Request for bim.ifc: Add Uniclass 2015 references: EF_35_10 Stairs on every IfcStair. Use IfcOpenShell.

First a look at what the model holds.

```python
import ifcopenshell

model = ifcopenshell.open("bim.ifc")
print(model.schema)
print("classifications:", [c.Name for c in model.by_type("IfcClassification")])
for ifc_class in ("IfcDoor", "IfcRoof", "IfcStair", "IfcWall", "IfcWindow"):
    print(ifc_class, len(model.by_type(ifc_class)))
```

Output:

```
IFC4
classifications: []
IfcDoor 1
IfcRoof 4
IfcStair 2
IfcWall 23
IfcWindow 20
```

```python
import ifcopenshell
import ifcopenshell.api.classification

model = ifcopenshell.open("bim.ifc")

system = ifcopenshell.api.classification.add_classification(model, classification="Uniclass 2015")

codes = {
    "IfcStair": ("EF_35_10", "Stairs"),
}
for ifc_class, (code, name) in codes.items():
    products = model.by_type(ifc_class)
    ifcopenshell.api.classification.add_reference(
        model, products=products, classification=system, identification=code, name=name
    )
    print(code, len(products))

model.write("bim_v2.ifc")
```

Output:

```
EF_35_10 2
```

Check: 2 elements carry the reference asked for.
